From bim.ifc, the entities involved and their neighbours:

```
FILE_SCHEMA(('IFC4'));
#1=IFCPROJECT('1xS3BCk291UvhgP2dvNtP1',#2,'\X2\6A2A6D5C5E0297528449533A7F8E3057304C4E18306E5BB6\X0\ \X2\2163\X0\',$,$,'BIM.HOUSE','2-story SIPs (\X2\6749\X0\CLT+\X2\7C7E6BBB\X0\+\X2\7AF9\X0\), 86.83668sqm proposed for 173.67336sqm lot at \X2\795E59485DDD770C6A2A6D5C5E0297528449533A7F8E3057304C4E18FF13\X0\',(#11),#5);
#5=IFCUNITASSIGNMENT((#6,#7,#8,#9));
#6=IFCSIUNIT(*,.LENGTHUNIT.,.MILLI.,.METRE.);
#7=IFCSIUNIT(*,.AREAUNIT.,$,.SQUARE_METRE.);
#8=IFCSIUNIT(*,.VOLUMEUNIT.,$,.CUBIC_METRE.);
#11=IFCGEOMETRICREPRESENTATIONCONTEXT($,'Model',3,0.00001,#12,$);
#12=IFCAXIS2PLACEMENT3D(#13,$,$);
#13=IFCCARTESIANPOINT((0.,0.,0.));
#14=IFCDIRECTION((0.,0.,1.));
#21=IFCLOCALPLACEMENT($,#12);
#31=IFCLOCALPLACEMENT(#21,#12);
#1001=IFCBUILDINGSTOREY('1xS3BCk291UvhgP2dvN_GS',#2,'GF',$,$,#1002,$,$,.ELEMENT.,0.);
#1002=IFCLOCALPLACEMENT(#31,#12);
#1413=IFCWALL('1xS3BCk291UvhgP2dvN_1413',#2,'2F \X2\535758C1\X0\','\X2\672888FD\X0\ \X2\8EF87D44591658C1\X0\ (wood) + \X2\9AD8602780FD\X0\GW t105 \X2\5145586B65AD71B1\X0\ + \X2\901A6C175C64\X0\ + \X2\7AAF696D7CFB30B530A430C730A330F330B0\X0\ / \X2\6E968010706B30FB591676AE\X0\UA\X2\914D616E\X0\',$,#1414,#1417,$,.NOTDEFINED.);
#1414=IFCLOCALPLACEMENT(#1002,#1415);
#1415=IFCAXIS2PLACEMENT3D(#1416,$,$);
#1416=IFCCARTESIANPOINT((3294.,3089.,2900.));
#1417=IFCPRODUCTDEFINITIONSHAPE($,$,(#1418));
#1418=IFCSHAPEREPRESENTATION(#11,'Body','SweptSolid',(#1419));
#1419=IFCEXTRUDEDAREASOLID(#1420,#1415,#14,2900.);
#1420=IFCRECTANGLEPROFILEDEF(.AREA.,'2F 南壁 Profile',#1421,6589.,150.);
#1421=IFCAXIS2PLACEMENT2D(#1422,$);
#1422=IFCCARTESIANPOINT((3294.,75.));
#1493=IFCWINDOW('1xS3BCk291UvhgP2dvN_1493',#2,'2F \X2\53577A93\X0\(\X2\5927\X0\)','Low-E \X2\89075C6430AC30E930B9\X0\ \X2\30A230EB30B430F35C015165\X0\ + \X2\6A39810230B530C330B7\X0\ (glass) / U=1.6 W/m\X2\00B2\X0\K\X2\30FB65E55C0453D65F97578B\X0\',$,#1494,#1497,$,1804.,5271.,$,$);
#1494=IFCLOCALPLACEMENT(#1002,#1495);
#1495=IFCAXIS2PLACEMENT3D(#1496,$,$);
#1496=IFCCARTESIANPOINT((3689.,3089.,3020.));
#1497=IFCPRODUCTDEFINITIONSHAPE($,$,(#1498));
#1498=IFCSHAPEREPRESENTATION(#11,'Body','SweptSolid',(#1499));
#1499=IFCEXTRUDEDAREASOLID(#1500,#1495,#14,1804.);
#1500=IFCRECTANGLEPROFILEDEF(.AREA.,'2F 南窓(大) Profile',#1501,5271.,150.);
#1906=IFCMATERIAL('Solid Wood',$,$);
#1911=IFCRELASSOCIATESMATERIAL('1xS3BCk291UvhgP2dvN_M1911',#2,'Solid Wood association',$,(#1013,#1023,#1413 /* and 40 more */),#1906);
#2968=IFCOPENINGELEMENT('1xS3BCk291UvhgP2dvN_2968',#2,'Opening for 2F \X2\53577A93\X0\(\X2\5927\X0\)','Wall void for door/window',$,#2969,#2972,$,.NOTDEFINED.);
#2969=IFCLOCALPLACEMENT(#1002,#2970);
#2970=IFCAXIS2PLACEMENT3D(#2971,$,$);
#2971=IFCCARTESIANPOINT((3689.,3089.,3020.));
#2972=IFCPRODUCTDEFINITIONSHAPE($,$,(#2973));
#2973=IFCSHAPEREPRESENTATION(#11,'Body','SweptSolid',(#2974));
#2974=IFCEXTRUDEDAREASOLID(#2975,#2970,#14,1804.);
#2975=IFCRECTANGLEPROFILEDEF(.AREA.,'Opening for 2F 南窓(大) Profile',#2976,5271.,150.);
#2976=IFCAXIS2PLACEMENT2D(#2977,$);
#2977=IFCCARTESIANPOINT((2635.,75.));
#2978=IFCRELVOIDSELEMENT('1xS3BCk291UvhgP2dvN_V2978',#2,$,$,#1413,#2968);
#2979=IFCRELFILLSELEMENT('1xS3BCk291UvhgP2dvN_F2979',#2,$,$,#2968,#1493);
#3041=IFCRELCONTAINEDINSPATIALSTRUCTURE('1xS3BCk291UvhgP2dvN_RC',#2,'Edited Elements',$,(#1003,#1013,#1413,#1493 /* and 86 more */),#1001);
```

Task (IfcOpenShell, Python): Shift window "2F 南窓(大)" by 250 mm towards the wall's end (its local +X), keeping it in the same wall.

```python
import ifcopenshell
import ifcopenshell.api.geometry
import ifcopenshell.util.placement

model = ifcopenshell.open("bim.ifc")

window = model.by_guid("1xS3BCk291UvhgP2dvN_1493")
opening = window.FillsVoids[0].RelatingOpeningElement
wall = opening.VoidsElements[0].RelatingBuildingElement

wall_matrix = ifcopenshell.util.placement.get_local_placement(wall.ObjectPlacement)
shift = wall_matrix[:3, 0] * 250.0
before = ifcopenshell.util.placement.get_local_placement(window.ObjectPlacement)[:3, 3].copy()

# The window is not placed relative to its opening, so move both.
for product in (opening, window):
    matrix = ifcopenshell.util.placement.get_local_placement(product.ObjectPlacement)
    matrix[:3, 3] += shift
    ifcopenshell.api.geometry.edit_object_placement(model, product=product, matrix=matrix, is_si=False)

after = ifcopenshell.util.placement.get_local_placement(window.ObjectPlacement)[:3, 3]
print("window moved by", (after - before).round(3) + 0.0)

model.write("bim_rev.ifc")
```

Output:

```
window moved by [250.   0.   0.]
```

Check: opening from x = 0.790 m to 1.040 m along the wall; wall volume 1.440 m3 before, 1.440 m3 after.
